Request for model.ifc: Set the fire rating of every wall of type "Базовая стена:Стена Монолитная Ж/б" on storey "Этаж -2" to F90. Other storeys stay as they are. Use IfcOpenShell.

First a look at what the model holds.

```python
import ifcopenshell
import ifcopenshell.util.element

model = ifcopenshell.open("model.ifc")
print(model.schema)
storey = next(s for s in model.by_type("IfcBuildingStorey") if s.Name == "Этаж -2")
walls = [e for e in ifcopenshell.util.element.get_decomposition(storey) if e.is_a("IfcWall")]
seen = {}
for e in walls:
    element_type = ifcopenshell.util.element.get_type(e)
    key = (element_type.Name if element_type != e and element_type else None, ifcopenshell.util.element.get_pset(e, "Pset_WallCommon", "FireRating"))
    seen[key] = seen.get(key, 0) + 1
for (name, value), count in sorted(seen.items(), key=str):
    print(count, "x", name, "|", value)
```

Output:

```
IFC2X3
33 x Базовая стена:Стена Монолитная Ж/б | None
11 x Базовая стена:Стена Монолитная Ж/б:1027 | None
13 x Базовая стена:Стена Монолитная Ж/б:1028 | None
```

```python
import ifcopenshell
import ifcopenshell.api.pset
import ifcopenshell.util.element

model = ifcopenshell.open("model.ifc")

storey = next(s for s in model.by_type("IfcBuildingStorey") if s.Name == "Этаж -2")
walls = [e for e in ifcopenshell.util.element.get_decomposition(storey) if e.is_a("IfcWall")]

count = 0
for e in walls:
    element_type = ifcopenshell.util.element.get_type(e)
    if element_type in (None, e) or element_type.Name != "Базовая стена:Стена Монолитная Ж/б":
        continue
    # add_pset returns the element's existing set when there is one.
    pset = ifcopenshell.api.pset.add_pset(model, product=e, name="Pset_WallCommon")
    ifcopenshell.api.pset.edit_pset(model, pset=pset, properties={"FireRating": "F90"})
    count += 1

print(count, "walls updated")

model.write("model_updated.ifc")
```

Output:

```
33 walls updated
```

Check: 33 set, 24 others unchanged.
